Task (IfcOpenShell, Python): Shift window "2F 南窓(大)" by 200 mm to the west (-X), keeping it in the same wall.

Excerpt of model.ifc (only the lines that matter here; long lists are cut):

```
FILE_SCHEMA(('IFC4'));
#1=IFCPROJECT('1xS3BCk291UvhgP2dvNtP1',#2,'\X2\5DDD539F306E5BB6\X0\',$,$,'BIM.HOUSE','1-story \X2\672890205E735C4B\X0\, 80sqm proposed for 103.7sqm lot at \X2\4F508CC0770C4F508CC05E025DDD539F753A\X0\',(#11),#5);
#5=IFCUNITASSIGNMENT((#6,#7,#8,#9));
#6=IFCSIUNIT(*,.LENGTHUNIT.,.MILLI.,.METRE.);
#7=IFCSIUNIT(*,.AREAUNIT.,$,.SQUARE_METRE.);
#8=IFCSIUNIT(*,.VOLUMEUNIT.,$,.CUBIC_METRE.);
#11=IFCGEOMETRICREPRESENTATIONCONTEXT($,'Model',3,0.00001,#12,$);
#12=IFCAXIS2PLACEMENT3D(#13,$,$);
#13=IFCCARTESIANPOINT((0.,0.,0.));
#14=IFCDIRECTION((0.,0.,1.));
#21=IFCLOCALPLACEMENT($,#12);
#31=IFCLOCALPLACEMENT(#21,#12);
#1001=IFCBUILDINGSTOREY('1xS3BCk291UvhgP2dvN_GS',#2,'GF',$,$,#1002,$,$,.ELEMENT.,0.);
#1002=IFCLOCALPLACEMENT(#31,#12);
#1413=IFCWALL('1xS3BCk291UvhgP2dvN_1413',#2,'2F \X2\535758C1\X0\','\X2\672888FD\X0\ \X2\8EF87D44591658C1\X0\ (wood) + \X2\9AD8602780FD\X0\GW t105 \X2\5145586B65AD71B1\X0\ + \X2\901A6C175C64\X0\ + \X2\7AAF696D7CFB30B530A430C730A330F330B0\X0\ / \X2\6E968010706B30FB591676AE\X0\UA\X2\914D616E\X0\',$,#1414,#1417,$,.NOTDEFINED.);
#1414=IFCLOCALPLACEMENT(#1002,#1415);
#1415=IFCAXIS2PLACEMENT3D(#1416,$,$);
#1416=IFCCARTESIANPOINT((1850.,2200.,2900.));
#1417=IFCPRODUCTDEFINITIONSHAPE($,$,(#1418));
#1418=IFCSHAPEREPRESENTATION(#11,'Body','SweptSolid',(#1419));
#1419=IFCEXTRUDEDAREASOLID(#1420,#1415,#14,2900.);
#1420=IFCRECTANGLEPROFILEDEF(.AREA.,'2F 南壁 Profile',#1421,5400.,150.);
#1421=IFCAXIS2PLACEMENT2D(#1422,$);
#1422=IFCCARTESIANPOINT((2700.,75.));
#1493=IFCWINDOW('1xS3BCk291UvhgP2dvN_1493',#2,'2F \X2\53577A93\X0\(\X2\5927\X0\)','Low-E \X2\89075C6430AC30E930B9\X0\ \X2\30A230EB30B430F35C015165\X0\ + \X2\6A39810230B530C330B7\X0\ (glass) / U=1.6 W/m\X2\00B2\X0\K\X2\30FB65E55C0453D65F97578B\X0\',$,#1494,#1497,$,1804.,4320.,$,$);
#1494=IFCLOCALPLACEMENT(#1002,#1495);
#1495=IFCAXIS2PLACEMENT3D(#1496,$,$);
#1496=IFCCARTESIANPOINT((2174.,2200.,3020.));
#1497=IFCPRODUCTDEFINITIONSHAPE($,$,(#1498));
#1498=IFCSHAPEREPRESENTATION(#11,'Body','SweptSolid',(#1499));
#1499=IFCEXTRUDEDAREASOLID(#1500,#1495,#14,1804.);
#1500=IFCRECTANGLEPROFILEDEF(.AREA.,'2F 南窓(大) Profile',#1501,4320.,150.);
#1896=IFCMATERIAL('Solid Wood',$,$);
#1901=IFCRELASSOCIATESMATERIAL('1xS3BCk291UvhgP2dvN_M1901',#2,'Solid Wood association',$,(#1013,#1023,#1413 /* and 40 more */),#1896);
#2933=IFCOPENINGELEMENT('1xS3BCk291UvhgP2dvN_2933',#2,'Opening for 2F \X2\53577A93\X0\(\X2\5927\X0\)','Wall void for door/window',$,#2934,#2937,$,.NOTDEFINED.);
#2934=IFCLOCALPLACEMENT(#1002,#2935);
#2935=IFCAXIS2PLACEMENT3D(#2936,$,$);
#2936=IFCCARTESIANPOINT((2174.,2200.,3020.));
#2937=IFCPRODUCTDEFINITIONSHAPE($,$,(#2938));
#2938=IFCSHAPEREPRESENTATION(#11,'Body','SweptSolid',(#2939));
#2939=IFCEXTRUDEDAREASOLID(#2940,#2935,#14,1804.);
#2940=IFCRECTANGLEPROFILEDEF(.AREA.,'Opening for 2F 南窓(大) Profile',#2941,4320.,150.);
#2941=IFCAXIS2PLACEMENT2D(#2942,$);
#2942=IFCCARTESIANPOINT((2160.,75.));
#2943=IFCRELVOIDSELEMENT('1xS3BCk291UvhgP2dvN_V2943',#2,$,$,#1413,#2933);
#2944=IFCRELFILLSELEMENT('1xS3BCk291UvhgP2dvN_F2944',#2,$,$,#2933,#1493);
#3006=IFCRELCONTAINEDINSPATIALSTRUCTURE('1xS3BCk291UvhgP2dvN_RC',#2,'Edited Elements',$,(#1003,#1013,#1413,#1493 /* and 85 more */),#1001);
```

```python
import ifcopenshell
import ifcopenshell.api.geometry
import ifcopenshell.util.placement
import ifcopenshell.util.unit

model = ifcopenshell.open("model.ifc")
unit_scale = ifcopenshell.util.unit.calculate_unit_scale(model)

window = model.by_guid("1xS3BCk291UvhgP2dvN_1493")
opening = window.FillsVoids[0].RelatingOpeningElement
wall = opening.VoidsElements[0].RelatingBuildingElement

wall_matrix = ifcopenshell.util.placement.get_local_placement(wall.ObjectPlacement)
shift = wall_matrix[:3, 0] * -0.2 / unit_scale
before = ifcopenshell.util.placement.get_local_placement(window.ObjectPlacement)[:3, 3].copy()

# The window is not placed relative to its opening, so move both.
for product in (opening, window):
    matrix = ifcopenshell.util.placement.get_local_placement(product.ObjectPlacement)
    matrix[:3, 3] += shift
    ifcopenshell.api.geometry.edit_object_placement(model, product=product, matrix=matrix, is_si=False)

after = ifcopenshell.util.placement.get_local_placement(window.ObjectPlacement)[:3, 3]
print("window moved by", (after - before).round(3) + 0.0)

model.write("model-out.ifc")
```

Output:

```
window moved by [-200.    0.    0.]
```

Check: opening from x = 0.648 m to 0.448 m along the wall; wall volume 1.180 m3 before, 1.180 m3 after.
